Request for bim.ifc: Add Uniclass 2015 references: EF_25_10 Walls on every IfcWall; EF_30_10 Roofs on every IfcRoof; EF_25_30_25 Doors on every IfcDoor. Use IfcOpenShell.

First a look at what the model holds.

```python
import ifcopenshell

model = ifcopenshell.open("bim.ifc")
print(model.schema)
print("classifications:", [c.Name for c in model.by_type("IfcClassification")])
for ifc_class in ("IfcDoor", "IfcRoof", "IfcStair", "IfcWall", "IfcWindow"):
    print(ifc_class, len(model.by_type(ifc_class)))
```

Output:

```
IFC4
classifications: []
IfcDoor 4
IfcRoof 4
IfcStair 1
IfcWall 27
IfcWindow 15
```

```python
import ifcopenshell
import ifcopenshell.api.classification

model = ifcopenshell.open("bim.ifc")

system = ifcopenshell.api.classification.add_classification(model, classification="Uniclass 2015")

codes = {
    "IfcWall": ("EF_25_10", "Walls"),
    "IfcRoof": ("EF_30_10", "Roofs"),
    "IfcDoor": ("EF_25_30_25", "Doors"),
}
for ifc_class, (code, name) in codes.items():
    products = model.by_type(ifc_class)
    ifcopenshell.api.classification.add_reference(
        model, products=products, classification=system, identification=code, name=name
    )
    print(code, len(products))

model.write("bim-out.ifc")
```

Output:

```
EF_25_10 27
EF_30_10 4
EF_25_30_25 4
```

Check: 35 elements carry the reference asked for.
